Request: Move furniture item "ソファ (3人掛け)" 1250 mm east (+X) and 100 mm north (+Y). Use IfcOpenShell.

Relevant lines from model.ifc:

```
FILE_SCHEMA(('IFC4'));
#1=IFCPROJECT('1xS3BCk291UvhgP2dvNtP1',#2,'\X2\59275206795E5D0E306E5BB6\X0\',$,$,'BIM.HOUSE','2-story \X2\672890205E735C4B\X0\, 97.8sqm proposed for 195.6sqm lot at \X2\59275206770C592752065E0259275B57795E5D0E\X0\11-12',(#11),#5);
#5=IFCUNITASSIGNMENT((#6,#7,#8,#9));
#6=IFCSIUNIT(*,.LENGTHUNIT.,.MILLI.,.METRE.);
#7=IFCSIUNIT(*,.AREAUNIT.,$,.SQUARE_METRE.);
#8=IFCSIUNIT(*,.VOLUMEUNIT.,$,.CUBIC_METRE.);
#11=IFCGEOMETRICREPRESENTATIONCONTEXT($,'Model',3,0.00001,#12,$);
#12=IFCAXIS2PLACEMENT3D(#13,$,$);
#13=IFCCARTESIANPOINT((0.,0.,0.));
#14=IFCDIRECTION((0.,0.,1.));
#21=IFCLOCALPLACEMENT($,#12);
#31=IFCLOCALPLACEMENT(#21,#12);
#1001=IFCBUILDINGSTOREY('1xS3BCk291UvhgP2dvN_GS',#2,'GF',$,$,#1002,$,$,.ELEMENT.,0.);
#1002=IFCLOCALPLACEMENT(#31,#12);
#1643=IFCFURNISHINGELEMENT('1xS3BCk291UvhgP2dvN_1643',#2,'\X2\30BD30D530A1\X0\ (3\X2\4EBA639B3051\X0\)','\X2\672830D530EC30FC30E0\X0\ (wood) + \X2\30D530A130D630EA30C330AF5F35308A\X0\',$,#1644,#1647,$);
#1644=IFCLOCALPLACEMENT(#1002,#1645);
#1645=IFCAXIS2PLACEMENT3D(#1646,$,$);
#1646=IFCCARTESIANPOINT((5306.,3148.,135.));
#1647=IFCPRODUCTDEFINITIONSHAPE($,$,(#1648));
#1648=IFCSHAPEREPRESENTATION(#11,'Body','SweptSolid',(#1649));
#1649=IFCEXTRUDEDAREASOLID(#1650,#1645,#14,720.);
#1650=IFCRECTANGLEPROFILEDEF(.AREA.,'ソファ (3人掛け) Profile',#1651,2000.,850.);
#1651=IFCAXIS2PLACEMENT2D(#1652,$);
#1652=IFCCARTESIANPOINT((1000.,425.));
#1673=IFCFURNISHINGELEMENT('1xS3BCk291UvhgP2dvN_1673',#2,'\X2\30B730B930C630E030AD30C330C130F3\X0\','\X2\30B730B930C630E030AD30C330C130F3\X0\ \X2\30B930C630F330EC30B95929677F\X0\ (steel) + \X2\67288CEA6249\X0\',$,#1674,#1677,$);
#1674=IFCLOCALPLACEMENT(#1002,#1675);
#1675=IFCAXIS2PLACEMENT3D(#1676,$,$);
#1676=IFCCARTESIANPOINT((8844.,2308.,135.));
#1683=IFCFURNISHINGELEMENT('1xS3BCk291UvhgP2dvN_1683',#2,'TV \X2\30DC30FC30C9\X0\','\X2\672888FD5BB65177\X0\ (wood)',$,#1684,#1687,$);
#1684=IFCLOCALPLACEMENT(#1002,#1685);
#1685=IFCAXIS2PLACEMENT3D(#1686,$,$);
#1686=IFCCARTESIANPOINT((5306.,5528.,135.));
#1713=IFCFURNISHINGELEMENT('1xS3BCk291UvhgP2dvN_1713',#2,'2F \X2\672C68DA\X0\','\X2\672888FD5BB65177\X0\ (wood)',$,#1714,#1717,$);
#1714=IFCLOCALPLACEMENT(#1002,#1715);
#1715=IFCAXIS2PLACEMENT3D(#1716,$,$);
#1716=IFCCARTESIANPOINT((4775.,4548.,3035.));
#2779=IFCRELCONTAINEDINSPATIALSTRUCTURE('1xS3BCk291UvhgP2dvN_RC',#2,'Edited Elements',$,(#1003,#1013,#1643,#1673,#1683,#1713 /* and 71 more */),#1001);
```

```python
import ifcopenshell
import ifcopenshell.api.geometry
import ifcopenshell.util.placement
import ifcopenshell.util.unit

model = ifcopenshell.open("model.ifc")
unit_scale = ifcopenshell.util.unit.calculate_unit_scale(model)

item = model.by_id(1643)
matrix = ifcopenshell.util.placement.get_local_placement(item.ObjectPlacement)
matrix[0, 3] += 1.25 / unit_scale
matrix[1, 3] += 0.1 / unit_scale
ifcopenshell.api.geometry.edit_object_placement(model, product=item, matrix=matrix, is_si=False)

print(ifcopenshell.util.placement.get_local_placement(item.ObjectPlacement).round(3) + 0.0)

model.write("model_v2.ifc")
```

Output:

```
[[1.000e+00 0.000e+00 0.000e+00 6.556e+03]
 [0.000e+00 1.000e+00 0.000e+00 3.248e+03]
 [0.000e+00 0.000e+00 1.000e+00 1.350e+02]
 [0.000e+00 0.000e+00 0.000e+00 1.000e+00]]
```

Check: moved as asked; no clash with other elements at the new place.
